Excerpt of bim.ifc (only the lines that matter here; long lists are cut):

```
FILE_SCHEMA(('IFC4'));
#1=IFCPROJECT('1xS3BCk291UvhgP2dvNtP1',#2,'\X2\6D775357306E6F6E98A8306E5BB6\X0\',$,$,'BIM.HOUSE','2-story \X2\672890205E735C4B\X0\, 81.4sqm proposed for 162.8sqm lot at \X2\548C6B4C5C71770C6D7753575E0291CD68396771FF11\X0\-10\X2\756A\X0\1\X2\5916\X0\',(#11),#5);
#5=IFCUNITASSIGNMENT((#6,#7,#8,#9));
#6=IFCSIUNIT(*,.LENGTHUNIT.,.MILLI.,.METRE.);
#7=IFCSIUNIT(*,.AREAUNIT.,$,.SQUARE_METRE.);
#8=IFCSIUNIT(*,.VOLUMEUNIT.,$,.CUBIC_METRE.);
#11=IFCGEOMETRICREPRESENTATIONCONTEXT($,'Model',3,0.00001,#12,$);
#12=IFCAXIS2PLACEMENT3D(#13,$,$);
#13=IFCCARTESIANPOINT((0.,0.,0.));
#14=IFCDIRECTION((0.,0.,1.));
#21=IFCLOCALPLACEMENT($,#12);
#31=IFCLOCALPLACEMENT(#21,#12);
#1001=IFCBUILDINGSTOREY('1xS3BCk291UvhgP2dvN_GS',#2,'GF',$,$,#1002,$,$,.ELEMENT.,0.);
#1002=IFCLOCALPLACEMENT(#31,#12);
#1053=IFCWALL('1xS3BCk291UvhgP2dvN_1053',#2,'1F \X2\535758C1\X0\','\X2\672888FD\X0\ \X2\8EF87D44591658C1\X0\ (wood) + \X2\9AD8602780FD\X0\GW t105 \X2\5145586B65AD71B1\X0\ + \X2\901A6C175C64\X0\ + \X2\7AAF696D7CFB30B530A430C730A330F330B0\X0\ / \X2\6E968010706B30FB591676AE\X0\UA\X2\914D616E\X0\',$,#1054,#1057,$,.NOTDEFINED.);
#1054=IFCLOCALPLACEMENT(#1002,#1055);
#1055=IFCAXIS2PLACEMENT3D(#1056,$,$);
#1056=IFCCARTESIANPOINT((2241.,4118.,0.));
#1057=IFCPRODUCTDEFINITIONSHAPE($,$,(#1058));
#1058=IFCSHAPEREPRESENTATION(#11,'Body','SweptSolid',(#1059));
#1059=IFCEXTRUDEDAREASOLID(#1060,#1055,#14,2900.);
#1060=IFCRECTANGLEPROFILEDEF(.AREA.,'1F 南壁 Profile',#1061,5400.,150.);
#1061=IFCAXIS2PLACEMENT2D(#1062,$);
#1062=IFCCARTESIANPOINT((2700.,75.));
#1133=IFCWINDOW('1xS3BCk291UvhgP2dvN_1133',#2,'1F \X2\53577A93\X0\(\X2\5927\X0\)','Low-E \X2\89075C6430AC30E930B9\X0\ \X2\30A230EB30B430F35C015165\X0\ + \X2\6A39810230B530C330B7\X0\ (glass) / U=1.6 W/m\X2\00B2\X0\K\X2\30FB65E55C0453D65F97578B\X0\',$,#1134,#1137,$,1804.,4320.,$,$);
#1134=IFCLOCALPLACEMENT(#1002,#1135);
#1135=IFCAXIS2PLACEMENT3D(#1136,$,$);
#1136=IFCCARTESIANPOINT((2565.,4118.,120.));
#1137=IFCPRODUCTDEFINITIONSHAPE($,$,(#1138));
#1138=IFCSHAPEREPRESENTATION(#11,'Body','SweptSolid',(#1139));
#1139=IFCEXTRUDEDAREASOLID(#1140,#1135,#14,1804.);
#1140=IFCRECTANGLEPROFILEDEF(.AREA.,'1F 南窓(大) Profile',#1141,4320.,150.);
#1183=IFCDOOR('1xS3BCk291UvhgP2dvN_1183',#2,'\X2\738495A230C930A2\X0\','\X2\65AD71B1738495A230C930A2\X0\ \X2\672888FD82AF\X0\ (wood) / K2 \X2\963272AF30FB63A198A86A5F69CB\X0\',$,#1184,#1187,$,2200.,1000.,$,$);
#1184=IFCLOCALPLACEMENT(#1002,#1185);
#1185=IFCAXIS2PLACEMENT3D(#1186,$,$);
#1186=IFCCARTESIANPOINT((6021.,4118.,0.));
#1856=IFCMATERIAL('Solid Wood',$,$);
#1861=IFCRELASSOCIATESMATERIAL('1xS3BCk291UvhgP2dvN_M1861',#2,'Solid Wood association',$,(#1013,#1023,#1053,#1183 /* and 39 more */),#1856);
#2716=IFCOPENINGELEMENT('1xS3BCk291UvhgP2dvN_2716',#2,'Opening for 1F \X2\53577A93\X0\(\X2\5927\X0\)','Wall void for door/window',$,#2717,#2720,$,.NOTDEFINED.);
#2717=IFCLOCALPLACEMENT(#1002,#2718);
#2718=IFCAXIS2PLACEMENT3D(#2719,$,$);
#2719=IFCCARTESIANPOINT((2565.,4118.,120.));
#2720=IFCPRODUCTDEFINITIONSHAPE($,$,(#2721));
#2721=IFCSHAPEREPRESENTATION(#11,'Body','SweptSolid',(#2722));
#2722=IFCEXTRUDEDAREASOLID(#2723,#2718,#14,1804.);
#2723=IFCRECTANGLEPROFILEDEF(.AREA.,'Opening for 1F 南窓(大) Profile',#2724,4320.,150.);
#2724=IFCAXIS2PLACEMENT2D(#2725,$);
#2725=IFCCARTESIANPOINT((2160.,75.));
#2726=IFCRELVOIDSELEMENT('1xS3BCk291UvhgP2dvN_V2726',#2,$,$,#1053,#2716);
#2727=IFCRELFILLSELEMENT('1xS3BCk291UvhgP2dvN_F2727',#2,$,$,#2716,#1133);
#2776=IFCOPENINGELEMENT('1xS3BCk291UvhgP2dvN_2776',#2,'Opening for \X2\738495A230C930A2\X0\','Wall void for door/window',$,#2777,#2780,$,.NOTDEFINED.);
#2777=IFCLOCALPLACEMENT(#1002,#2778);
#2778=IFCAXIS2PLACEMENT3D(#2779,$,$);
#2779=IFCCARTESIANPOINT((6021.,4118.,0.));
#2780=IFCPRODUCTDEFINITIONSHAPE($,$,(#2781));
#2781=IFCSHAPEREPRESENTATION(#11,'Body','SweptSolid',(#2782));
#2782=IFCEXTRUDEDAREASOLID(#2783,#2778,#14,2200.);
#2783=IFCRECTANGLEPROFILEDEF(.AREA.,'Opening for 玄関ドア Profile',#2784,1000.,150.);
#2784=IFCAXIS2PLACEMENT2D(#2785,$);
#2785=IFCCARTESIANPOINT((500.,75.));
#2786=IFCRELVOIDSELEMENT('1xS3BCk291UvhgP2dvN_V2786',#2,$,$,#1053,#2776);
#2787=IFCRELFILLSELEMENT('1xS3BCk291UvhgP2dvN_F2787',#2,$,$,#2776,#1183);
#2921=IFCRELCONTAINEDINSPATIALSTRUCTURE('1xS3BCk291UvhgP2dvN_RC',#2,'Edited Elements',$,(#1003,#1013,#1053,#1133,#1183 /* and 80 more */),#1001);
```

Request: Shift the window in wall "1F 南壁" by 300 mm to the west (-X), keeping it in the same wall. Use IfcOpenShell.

```python
import ifcopenshell
import ifcopenshell.api.geometry
import ifcopenshell.util.placement
import ifcopenshell.util.unit

model = ifcopenshell.open("bim.ifc")
unit_scale = ifcopenshell.util.unit.calculate_unit_scale(model)

window = model.by_guid("1xS3BCk291UvhgP2dvN_1133")
opening = window.FillsVoids[0].RelatingOpeningElement
wall = opening.VoidsElements[0].RelatingBuildingElement

wall_matrix = ifcopenshell.util.placement.get_local_placement(wall.ObjectPlacement)
shift = wall_matrix[:3, 0] * -0.3 / unit_scale
before = ifcopenshell.util.placement.get_local_placement(window.ObjectPlacement)[:3, 3].copy()

# The window is not placed relative to its opening, so move both.
for product in (opening, window):
    matrix = ifcopenshell.util.placement.get_local_placement(product.ObjectPlacement)
    matrix[:3, 3] += shift
    ifcopenshell.api.geometry.edit_object_placement(model, product=product, matrix=matrix, is_si=False)

after = ifcopenshell.util.placement.get_local_placement(window.ObjectPlacement)[:3, 3]
print("window moved by", (after - before).round(3) + 0.0)

model.write("bim_rev.ifc")
```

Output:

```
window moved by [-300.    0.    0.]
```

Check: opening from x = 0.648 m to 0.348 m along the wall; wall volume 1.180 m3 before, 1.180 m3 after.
